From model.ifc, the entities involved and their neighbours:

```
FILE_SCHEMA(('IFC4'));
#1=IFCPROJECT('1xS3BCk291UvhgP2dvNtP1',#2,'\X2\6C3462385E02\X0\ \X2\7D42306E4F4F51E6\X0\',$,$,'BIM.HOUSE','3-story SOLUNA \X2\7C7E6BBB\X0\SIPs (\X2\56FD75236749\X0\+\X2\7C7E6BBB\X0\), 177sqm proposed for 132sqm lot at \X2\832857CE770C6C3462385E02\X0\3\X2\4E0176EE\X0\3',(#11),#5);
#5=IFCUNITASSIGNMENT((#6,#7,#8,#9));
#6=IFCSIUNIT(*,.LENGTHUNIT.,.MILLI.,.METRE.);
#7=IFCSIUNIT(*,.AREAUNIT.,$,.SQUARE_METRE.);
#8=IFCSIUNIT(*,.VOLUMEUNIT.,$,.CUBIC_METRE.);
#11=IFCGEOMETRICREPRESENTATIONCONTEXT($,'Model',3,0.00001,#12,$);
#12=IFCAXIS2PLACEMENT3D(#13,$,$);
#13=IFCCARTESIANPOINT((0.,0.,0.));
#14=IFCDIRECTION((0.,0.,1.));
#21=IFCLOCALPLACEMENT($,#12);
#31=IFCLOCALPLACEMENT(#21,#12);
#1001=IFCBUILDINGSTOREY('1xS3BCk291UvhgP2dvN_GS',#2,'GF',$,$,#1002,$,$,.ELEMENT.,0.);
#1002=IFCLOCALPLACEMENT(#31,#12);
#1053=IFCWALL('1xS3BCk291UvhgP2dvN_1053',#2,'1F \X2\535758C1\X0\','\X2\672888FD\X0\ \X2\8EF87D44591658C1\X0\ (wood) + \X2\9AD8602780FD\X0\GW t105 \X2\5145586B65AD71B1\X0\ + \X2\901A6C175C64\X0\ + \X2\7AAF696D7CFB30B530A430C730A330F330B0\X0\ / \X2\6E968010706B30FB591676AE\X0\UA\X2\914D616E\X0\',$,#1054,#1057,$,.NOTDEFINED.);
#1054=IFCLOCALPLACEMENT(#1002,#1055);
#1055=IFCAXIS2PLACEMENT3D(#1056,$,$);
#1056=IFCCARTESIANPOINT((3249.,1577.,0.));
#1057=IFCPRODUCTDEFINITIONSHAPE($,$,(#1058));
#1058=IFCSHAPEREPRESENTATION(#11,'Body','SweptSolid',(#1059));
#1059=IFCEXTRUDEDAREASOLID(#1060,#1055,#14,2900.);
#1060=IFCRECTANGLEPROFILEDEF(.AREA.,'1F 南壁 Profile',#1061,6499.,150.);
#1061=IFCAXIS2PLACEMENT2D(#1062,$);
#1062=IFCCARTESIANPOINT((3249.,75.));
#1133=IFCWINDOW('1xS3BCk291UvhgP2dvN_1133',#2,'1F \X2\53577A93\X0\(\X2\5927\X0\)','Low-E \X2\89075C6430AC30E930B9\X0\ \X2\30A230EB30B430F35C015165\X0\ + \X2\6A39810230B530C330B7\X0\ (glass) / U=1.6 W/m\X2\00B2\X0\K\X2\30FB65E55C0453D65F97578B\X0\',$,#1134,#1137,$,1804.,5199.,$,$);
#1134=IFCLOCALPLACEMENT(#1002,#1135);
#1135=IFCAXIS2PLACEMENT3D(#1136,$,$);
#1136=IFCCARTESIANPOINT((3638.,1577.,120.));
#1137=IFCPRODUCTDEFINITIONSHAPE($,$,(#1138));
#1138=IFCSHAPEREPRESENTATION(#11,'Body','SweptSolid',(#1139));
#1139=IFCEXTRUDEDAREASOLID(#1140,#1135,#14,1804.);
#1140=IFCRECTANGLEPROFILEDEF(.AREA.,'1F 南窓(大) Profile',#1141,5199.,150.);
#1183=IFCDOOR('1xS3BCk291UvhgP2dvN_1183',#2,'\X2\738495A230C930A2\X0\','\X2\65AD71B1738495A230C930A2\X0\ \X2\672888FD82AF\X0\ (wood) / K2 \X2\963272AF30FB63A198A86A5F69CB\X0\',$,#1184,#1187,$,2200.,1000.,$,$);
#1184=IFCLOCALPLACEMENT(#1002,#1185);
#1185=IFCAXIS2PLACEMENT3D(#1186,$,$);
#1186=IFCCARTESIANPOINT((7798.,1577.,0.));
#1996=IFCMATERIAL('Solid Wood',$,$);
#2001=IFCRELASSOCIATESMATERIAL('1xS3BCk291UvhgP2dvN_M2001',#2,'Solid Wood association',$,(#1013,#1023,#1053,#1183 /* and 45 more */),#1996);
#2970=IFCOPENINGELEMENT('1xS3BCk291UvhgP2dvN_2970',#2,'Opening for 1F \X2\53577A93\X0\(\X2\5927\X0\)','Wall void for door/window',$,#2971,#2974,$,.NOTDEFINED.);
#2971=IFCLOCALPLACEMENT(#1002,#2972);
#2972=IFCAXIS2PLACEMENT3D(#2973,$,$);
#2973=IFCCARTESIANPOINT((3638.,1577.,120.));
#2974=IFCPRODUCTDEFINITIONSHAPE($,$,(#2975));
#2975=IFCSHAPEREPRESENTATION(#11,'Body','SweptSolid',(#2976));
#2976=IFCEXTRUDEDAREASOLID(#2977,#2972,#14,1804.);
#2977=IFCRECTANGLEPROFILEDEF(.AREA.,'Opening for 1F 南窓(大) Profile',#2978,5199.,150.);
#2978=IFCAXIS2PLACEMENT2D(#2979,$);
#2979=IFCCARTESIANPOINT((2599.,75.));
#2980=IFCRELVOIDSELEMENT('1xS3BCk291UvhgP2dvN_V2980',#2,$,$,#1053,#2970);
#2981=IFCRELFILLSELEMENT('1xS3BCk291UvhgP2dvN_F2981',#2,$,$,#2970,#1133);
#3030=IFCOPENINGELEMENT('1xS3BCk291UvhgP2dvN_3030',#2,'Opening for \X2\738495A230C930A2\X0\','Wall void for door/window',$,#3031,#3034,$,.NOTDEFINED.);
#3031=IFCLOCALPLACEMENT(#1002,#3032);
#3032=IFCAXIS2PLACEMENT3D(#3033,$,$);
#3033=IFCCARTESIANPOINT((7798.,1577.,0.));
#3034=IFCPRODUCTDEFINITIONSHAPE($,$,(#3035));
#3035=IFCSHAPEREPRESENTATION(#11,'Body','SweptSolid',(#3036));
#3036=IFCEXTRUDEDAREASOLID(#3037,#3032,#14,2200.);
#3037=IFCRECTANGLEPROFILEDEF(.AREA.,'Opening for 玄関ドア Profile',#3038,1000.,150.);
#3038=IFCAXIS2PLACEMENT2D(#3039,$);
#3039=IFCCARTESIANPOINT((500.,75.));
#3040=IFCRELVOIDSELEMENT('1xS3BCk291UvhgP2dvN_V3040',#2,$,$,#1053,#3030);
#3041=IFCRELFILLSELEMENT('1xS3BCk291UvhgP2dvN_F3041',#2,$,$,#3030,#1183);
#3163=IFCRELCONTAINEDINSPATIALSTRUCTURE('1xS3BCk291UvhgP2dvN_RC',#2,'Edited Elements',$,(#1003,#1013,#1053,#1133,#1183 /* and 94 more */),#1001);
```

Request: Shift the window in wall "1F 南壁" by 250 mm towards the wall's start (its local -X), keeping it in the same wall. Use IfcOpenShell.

```python
import ifcopenshell
import ifcopenshell.api.geometry
import ifcopenshell.util.placement
import ifcopenshell.util.unit

model = ifcopenshell.open("model.ifc")
unit_scale = ifcopenshell.util.unit.calculate_unit_scale(model)

window = model.by_guid("1xS3BCk291UvhgP2dvN_1133")
opening = window.FillsVoids[0].RelatingOpeningElement
wall = opening.VoidsElements[0].RelatingBuildingElement

wall_matrix = ifcopenshell.util.placement.get_local_placement(wall.ObjectPlacement)
shift = wall_matrix[:3, 0] * -0.25 / unit_scale
before = ifcopenshell.util.placement.get_local_placement(window.ObjectPlacement)[:3, 3].copy()

# The window is not placed relative to its opening, so move both.
for product in (opening, window):
    matrix = ifcopenshell.util.placement.get_local_placement(product.ObjectPlacement)
    matrix[:3, 3] += shift
    ifcopenshell.api.geometry.edit_object_placement(model, product=product, matrix=matrix, is_si=False)

after = ifcopenshell.util.placement.get_local_placement(window.ObjectPlacement)[:3, 3]
print("window moved by", (after - before).round(3) + 0.0)

model.write("model_updated.ifc")
```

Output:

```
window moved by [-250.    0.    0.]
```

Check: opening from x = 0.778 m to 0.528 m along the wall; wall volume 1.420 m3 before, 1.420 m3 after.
